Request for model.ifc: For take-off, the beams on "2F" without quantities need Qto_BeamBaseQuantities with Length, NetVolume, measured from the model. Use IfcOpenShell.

First a look at what the model holds.

```python
import ifcopenshell
import ifcopenshell.util.element
import ifcopenshell.util.unit

model = ifcopenshell.open("model.ifc")
print(model.schema)
for unit_type in ("LENGTHUNIT", "AREAUNIT", "VOLUMEUNIT"):
    print(unit_type, ifcopenshell.util.unit.calculate_unit_scale(model, unit_type))
storey = next(s for s in model.by_type("IfcBuildingStorey") if s.Name == "2F")
beams = [e for e in ifcopenshell.util.element.get_decomposition(storey) if e.is_a("IfcBeam")]
for e in sorted(beams, key=lambda e: e.id()):
    print(e.id(), e.is_a(), e.Name, list(ifcopenshell.util.element.get_psets(e, qtos_only=True)), sep=" | ")
```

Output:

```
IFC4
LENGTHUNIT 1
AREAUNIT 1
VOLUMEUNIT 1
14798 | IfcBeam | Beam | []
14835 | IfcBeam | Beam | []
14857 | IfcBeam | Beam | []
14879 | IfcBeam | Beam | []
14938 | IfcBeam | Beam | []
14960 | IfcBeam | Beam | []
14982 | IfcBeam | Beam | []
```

```python
import ifcopenshell
import ifcopenshell.api.pset
import ifcopenshell.geom
import ifcopenshell.util.element
import ifcopenshell.util.shape
import ifcopenshell.util.unit

model = ifcopenshell.open("model.ifc")
unit_scale = ifcopenshell.util.unit.calculate_unit_scale(model)
volume_scale = ifcopenshell.util.unit.calculate_unit_scale(model, "VOLUMEUNIT")
settings = ifcopenshell.geom.settings()

storey = next(s for s in model.by_type("IfcBuildingStorey") if s.Name == "2F")
beams = [e for e in ifcopenshell.util.element.get_decomposition(storey) if e.is_a("IfcBeam")]

for e in sorted(beams, key=lambda e: e.id()):
    if ifcopenshell.util.element.get_psets(e, qtos_only=True, should_inherit=False):
        continue
    # Geometry comes back in metres, in the element's own axes.
    shape = ifcopenshell.geom.create_shape(settings, e)
    values = {
        "Length": ifcopenshell.util.shape.get_max_xyz(shape.geometry) / unit_scale,
        "NetVolume": ifcopenshell.util.shape.get_volume(shape.geometry) / volume_scale,
    }
    qto = ifcopenshell.api.pset.add_qto(model, product=e, name="Qto_BeamBaseQuantities")
    ifcopenshell.api.pset.edit_qto(model, qto=qto, properties=values)
    print(e.id(), {k: round(v, 3) for k, v in values.items()})

model.write("model_updated.ifc")
```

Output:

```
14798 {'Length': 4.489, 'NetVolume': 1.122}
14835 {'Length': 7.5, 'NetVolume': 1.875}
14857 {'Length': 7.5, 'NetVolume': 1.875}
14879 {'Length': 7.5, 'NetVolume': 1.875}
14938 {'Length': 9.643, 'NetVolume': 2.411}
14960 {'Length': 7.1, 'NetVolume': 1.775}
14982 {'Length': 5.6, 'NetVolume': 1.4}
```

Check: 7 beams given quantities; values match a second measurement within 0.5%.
